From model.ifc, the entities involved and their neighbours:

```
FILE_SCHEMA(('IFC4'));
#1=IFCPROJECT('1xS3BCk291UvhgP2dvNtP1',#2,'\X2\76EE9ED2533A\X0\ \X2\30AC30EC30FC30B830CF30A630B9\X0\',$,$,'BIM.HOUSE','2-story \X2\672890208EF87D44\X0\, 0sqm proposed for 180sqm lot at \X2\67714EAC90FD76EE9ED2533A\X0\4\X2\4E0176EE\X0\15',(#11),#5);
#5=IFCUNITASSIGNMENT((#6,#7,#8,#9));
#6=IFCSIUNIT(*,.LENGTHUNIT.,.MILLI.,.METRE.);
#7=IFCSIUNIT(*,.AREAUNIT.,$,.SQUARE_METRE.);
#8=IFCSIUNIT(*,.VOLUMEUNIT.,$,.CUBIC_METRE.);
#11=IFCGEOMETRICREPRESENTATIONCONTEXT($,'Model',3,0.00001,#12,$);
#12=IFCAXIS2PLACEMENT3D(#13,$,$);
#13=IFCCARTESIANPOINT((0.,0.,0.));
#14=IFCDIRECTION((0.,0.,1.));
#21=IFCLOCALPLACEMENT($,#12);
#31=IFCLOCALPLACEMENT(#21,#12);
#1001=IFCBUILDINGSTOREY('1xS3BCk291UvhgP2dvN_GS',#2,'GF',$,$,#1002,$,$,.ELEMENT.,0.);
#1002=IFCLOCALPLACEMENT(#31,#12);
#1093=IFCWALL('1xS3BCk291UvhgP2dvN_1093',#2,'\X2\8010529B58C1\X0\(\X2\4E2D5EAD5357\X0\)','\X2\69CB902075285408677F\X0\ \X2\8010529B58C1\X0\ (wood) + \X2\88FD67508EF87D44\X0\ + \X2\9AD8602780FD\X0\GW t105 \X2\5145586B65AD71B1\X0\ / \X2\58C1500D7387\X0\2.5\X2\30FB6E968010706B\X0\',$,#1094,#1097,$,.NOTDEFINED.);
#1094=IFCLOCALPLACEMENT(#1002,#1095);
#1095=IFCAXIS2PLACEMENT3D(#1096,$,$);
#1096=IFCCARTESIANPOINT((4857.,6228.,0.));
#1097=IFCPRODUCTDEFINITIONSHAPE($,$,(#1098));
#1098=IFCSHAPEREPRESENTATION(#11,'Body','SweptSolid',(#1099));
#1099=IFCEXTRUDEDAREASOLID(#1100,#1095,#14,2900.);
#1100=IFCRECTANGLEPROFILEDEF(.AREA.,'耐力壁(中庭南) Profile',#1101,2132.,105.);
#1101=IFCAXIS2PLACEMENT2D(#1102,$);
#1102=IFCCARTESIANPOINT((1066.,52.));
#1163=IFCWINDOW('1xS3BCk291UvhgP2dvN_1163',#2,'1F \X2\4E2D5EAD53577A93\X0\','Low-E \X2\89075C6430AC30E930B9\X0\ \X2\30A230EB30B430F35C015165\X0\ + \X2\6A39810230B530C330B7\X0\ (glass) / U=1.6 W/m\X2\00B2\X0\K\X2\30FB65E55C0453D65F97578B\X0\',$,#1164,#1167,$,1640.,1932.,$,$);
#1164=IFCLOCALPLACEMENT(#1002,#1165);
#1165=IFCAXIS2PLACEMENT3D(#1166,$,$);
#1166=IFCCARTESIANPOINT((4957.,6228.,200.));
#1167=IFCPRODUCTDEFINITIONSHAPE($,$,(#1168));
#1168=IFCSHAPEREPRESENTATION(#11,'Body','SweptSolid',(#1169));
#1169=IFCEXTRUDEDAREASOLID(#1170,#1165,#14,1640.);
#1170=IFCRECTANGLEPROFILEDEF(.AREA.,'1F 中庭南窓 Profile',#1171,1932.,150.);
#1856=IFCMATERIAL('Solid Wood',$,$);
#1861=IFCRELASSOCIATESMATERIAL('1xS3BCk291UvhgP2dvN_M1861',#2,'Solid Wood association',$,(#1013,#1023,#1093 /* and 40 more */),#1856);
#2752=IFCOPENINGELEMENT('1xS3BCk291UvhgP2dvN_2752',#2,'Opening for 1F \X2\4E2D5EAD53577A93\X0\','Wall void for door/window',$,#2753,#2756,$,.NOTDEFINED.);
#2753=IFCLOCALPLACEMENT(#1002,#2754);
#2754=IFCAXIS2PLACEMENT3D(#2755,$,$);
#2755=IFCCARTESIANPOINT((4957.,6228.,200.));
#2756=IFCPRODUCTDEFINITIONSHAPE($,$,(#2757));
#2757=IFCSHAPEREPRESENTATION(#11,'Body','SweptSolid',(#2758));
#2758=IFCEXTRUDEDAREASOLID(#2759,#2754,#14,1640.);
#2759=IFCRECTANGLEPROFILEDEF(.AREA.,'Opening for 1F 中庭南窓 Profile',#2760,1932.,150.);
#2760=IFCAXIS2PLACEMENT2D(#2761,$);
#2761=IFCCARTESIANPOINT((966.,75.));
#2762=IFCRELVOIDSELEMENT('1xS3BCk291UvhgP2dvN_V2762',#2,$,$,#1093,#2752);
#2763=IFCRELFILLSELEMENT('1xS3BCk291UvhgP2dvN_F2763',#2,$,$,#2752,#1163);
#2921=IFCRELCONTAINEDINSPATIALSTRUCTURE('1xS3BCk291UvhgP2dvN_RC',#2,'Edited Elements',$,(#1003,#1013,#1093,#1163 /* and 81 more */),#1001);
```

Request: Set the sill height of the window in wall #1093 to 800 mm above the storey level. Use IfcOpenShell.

```python
import numpy as np
import ifcopenshell
import ifcopenshell.api.geometry
import ifcopenshell.geom
import ifcopenshell.util.element
import ifcopenshell.util.placement
import ifcopenshell.util.shape
import ifcopenshell.util.unit

model = ifcopenshell.open("model.ifc")
unit_scale = ifcopenshell.util.unit.calculate_unit_scale(model)

window = model.by_guid("1xS3BCk291UvhgP2dvN_1163")
opening = window.FillsVoids[0].RelatingOpeningElement
storey = ifcopenshell.util.element.get_container(window, ifc_class="IfcBuildingStorey")
level = ifcopenshell.util.placement.get_local_placement(storey.ObjectPlacement)[2, 3]

# The opening's origin need not be at the sill, so measure its lowest point.
shape = ifcopenshell.geom.create_shape(ifcopenshell.geom.settings(), opening)
bottom = ifcopenshell.util.shape.get_shape_bottom_elevation(shape, shape.geometry) / unit_scale
dz = level + 0.8 / unit_scale - bottom

shift = np.array([0.0, 0.0, dz])
# The window is not placed relative to its opening, so move both.
for product in (opening, window):
    matrix = ifcopenshell.util.placement.get_local_placement(product.ObjectPlacement)
    matrix[:3, 3] += shift
    ifcopenshell.api.geometry.edit_object_placement(model, product=product, matrix=matrix, is_si=False)

print(f"moved by {dz * unit_scale:+.3f} m")

model.write("model_v2.ifc")
```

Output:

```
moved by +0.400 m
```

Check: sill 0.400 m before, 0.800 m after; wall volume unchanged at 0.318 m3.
